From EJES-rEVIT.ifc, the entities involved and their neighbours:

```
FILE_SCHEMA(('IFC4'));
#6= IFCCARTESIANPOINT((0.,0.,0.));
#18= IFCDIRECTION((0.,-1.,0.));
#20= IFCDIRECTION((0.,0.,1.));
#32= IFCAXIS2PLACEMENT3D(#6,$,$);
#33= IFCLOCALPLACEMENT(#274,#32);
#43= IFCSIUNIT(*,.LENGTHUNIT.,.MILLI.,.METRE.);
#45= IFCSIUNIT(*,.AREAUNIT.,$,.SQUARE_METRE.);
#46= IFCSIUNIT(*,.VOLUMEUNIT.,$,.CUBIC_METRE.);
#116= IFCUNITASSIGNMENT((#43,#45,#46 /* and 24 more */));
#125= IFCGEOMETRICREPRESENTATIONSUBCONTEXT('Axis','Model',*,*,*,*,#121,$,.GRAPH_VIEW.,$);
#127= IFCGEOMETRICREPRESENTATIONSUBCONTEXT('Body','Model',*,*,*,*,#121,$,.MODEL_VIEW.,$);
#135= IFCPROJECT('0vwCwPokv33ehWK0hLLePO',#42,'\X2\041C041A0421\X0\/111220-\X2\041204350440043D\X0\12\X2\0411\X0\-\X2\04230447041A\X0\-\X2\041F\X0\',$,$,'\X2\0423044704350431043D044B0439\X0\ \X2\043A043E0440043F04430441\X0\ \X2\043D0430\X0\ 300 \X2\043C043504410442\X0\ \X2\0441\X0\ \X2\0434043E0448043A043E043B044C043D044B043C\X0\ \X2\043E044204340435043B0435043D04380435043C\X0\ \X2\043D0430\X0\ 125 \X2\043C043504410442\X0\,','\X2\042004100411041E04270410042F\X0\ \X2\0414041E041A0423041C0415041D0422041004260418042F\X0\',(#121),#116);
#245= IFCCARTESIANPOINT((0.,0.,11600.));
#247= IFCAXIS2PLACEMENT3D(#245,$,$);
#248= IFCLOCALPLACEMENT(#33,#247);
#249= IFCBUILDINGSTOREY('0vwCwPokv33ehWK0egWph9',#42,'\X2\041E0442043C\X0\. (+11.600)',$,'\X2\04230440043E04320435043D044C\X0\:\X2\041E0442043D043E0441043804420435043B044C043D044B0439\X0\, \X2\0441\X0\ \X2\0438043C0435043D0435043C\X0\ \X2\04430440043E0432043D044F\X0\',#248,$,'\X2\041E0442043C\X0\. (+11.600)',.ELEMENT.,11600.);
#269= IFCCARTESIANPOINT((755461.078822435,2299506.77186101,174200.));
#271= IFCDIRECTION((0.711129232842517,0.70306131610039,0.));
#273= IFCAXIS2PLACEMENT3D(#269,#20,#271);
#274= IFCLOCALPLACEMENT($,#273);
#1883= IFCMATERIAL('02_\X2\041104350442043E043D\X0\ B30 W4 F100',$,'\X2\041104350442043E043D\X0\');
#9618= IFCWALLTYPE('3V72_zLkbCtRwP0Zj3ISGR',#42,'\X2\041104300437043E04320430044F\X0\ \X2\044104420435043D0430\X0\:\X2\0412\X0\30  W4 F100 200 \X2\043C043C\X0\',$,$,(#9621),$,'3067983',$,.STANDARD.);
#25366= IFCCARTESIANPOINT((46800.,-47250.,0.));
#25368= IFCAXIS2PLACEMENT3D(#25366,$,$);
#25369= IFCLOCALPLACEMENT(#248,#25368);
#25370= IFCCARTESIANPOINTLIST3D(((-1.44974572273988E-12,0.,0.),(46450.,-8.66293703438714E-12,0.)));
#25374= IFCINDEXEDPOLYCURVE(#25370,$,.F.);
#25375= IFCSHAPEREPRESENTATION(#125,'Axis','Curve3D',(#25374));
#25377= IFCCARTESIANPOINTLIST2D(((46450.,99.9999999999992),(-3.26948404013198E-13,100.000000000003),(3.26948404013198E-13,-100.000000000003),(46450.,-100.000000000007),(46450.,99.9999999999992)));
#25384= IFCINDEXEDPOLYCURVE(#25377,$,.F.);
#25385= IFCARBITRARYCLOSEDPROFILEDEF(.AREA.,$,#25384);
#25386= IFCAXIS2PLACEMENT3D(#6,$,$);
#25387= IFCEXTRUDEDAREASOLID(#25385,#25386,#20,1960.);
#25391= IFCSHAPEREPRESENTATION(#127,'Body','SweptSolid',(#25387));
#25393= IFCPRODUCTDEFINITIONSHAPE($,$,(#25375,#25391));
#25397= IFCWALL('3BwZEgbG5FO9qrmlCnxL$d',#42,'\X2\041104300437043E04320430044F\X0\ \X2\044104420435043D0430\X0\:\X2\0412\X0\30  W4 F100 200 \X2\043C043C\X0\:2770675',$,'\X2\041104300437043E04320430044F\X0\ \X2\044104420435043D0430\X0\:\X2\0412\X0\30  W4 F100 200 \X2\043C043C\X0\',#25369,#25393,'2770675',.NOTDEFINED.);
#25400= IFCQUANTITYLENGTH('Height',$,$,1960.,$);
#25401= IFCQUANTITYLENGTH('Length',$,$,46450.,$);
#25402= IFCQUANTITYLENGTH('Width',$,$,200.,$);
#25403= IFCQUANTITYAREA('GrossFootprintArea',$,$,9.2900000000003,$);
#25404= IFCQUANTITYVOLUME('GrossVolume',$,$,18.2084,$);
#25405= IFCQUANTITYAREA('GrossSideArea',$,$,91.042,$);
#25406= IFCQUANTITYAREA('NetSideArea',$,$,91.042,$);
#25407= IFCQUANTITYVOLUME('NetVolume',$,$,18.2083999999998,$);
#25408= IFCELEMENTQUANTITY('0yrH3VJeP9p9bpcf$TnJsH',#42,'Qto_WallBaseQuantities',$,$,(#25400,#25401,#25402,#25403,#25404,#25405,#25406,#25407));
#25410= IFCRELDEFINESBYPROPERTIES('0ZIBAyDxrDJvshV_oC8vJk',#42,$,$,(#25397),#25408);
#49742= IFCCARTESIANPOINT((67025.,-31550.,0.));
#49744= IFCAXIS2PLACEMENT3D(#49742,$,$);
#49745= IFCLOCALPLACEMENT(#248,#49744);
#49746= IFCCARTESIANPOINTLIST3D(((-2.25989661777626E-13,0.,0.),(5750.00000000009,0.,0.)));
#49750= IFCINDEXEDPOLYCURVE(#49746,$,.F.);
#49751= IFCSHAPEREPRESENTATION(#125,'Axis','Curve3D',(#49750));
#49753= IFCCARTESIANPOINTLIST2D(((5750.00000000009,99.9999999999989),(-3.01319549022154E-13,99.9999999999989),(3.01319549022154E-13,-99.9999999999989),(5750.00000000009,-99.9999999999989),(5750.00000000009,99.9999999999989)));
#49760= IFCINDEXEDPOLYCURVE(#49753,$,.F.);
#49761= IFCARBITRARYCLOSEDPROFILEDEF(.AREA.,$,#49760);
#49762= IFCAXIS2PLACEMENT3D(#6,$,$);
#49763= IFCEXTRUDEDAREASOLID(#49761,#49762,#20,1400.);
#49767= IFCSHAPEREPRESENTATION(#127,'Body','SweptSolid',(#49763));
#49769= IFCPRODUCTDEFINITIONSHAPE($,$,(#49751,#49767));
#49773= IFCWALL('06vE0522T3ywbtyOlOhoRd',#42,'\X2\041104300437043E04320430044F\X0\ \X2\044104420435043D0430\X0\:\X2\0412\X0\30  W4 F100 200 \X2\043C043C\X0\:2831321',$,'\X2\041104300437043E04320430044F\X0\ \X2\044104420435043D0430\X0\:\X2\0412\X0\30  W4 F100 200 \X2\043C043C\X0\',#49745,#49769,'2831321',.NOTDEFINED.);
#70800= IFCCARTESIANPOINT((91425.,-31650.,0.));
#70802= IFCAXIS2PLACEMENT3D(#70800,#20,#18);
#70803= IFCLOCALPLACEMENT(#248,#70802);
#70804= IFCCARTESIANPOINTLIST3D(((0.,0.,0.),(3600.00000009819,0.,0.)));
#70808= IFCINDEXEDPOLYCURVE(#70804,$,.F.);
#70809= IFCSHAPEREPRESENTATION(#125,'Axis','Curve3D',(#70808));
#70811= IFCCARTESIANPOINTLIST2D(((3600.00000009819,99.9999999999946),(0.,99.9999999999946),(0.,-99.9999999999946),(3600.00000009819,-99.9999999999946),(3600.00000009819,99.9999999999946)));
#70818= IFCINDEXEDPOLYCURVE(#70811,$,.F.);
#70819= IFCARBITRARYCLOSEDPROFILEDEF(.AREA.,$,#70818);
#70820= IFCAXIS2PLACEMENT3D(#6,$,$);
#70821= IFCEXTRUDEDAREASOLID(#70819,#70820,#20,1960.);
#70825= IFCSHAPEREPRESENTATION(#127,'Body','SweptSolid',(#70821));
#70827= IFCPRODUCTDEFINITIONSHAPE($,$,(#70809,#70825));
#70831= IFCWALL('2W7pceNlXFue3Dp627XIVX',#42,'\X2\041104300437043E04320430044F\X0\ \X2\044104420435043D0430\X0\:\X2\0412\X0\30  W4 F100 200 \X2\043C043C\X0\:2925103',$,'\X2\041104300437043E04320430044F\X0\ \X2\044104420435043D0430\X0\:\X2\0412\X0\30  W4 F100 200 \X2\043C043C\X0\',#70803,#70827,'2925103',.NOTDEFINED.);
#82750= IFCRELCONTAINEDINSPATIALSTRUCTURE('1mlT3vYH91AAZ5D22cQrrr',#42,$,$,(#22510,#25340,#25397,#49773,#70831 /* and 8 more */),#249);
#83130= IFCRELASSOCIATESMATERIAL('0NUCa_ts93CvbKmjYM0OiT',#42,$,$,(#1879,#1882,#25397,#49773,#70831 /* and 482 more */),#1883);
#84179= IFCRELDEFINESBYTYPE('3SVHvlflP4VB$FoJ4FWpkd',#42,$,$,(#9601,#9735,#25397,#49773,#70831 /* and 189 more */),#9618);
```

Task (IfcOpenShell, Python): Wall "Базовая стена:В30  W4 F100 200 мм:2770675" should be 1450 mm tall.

```python
import ifcopenshell
import ifcopenshell.api.pset
import ifcopenshell.geom
import ifcopenshell.util.element
import ifcopenshell.util.representation
import ifcopenshell.util.shape
import ifcopenshell.util.unit

model = ifcopenshell.open("EJES-rEVIT.ifc")
unit_scale = ifcopenshell.util.unit.calculate_unit_scale(model)
area_scale = ifcopenshell.util.unit.calculate_unit_scale(model, "AREAUNIT")
volume_scale = ifcopenshell.util.unit.calculate_unit_scale(model, "VOLUMEUNIT")
settings = ifcopenshell.geom.settings()


def volume(element):
    """Net volume in cubic metres, openings subtracted."""
    shape = ifcopenshell.geom.create_shape(settings, element)
    return ifcopenshell.util.shape.get_volume(shape.geometry)


wall = model.by_guid("3BwZEgbG5FO9qrmlCnxL$d")
before = volume(wall)

body = ifcopenshell.util.representation.get_representation(wall, "Model", "Body")
solid = body.Items[0]
old_height = solid.Depth
solid.Depth = 1450.0
after = volume(wall)
thickness = 0.2  # wall thickness in metres

# Update the stored height, areas and volumes.
qto = model.by_id(ifcopenshell.util.element.get_pset(wall, "Qto_WallBaseQuantities", should_inherit=False)["id"])
ifcopenshell.api.pset.edit_qto(model, qto=qto, properties={
    "Height": solid.Depth,
    "GrossVolume": ifcopenshell.util.element.get_pset(wall, "Qto_WallBaseQuantities", "GrossVolume") * solid.Depth / old_height,
    "GrossSideArea": ifcopenshell.util.element.get_pset(wall, "Qto_WallBaseQuantities", "GrossSideArea") * solid.Depth / old_height,
    "NetSideArea": after / thickness / area_scale,
    "NetVolume": after / volume_scale,
})

print(f"height {old_height:g} -> {solid.Depth:g}, volume {before:.3f} -> {after:.3f} m3")

model.write("EJES-rEVIT_rev.ifc")
```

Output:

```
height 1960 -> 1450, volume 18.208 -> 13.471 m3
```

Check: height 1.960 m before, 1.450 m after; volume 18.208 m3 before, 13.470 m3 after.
